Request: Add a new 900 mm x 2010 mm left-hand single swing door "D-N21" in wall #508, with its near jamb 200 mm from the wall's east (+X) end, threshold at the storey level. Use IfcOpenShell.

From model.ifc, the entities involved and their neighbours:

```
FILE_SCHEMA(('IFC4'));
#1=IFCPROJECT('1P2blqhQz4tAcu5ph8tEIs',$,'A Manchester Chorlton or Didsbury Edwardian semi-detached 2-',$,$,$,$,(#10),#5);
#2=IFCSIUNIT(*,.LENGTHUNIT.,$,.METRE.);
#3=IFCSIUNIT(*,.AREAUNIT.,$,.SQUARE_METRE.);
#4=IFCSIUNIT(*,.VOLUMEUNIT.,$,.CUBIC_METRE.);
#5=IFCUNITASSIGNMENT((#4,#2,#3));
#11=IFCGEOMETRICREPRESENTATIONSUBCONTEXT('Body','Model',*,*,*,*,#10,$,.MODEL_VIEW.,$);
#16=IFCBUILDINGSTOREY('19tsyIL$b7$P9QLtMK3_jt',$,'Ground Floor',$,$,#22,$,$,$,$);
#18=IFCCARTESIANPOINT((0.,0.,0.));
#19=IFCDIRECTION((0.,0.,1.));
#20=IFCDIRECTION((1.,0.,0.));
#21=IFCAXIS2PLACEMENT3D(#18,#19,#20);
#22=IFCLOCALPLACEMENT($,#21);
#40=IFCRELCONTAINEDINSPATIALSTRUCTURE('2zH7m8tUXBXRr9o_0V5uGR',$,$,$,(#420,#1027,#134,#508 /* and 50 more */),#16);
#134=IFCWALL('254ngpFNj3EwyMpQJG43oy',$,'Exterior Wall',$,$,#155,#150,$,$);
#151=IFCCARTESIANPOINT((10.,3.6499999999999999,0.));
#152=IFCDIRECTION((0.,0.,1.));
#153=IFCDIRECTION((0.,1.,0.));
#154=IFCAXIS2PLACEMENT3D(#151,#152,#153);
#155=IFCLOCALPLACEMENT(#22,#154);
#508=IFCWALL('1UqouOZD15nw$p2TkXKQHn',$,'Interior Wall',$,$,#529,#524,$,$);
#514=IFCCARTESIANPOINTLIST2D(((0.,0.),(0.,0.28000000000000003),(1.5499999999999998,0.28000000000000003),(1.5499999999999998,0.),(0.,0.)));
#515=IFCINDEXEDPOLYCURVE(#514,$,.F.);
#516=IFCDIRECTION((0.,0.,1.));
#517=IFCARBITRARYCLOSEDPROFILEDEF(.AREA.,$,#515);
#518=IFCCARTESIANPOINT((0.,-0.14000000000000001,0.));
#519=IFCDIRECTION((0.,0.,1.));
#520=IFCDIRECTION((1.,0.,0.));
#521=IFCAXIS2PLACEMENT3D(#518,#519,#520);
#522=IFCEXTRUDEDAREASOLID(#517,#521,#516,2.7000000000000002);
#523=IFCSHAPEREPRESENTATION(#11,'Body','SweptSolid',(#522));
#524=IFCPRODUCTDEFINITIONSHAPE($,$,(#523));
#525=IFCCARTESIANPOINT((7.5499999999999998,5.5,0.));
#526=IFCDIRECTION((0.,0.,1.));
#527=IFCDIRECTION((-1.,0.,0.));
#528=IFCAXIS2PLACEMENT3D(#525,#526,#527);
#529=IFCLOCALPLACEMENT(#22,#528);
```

```python
import numpy as np
import ifcopenshell
import ifcopenshell.api.feature
import ifcopenshell.api.geometry
import ifcopenshell.api.root
import ifcopenshell.api.spatial
import ifcopenshell.geom
import ifcopenshell.util.element
import ifcopenshell.util.placement
import ifcopenshell.util.representation
import ifcopenshell.util.shape
import ifcopenshell.util.unit

model = ifcopenshell.open("model.ifc")
unit_scale = ifcopenshell.util.unit.calculate_unit_scale(model)
settings = ifcopenshell.geom.settings()


def volume(element):
    """Net volume in cubic metres, openings subtracted."""
    shape = ifcopenshell.geom.create_shape(settings, element)
    return ifcopenshell.util.shape.get_volume(shape.geometry)


wall = model.by_guid("1UqouOZD15nw$p2TkXKQHn")
storey = ifcopenshell.util.element.get_container(wall, ifc_class="IfcBuildingStorey")
context = ifcopenshell.util.representation.get_context(model, "Model", "Body", "MODEL_VIEW")
before = volume(wall)

width, height, from_end, sill = 0.9, 2.01, 0.2, 0.0  # metres

# The wall runs along its own X axis, and the end named is its -X end.
wall_shape = ifcopenshell.geom.create_shape(settings, wall)
x, y, z = ifcopenshell.util.shape.get_vertices(wall_shape.geometry).T
start = x.min() + from_end
face, thickness = float(y.min()), float(y.max() - y.min())
wall_matrix = ifcopenshell.util.placement.get_local_placement(wall.ObjectPlacement)
level = ifcopenshell.util.placement.get_local_placement(storey.ObjectPlacement)[2, 3]


def in_wall(x, y):
    """Placement at x, y metres in the wall's axes, at sill height."""
    matrix = wall_matrix.copy()
    matrix[:, 3] = wall_matrix @ np.array([x / unit_scale, y / unit_scale, 0.0, 1.0])
    matrix[2, 3] = level + sill / unit_scale
    return matrix


# Opening: a box that overshoots both wall faces by 50 mm.
opening = ifcopenshell.api.root.create_entity(model, ifc_class="IfcOpeningElement", predefined_type="OPENING")
box = ifcopenshell.api.geometry.add_wall_representation(
    model, context=context, length=width, height=height, thickness=thickness + 0.1
)
ifcopenshell.api.geometry.assign_representation(model, product=opening, representation=box)
ifcopenshell.api.geometry.edit_object_placement(model, product=opening, matrix=in_wall(start, face - 0.05), is_si=False)
ifcopenshell.api.feature.add_feature(model, feature=opening, element=wall)

door = ifcopenshell.api.root.create_entity(model, ifc_class="IfcDoor", name="D-N21", predefined_type="DOOR")
door.OverallWidth, door.OverallHeight = width / unit_scale, height / unit_scale
door.OperationType = "SINGLE_SWING_LEFT"
body = ifcopenshell.api.geometry.add_door_representation(
    model,
    context=context,
    overall_width=door.OverallWidth,
    overall_height=door.OverallHeight,
    operation_type="SINGLE_SWING_LEFT",
    lining_properties={"LiningDepth": thickness / unit_scale, "ThresholdDepth": thickness / unit_scale},
)
ifcopenshell.api.geometry.assign_representation(model, product=door, representation=body)
ifcopenshell.api.spatial.assign_container(model, products=[door], relating_structure=storey)
ifcopenshell.api.feature.add_filling(model, opening=opening, element=door)

# The lining spans the wall, so the door starts at the wall face.
ifcopenshell.api.geometry.edit_object_placement(model, product=door, matrix=in_wall(start, face), is_si=False)

after = volume(wall)

print(f"wall volume {before:.3f} -> {after:.3f} m3")

model.write("model_updated.ifc")
```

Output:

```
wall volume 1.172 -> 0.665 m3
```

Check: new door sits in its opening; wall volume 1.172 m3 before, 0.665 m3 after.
